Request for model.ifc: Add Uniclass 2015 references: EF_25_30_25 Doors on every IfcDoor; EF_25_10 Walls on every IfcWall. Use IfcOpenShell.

First a look at what the model holds.

```python
import ifcopenshell

model = ifcopenshell.open("model.ifc")
print(model.schema)
print("classifications:", [c.Name for c in model.by_type("IfcClassification")])
for ifc_class in ("IfcDoor", "IfcRoof", "IfcStair", "IfcWall", "IfcWindow"):
    print(ifc_class, len(model.by_type(ifc_class)))
```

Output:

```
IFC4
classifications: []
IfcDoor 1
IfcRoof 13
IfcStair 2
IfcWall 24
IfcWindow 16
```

```python
import ifcopenshell
import ifcopenshell.api.classification

model = ifcopenshell.open("model.ifc")

system = ifcopenshell.api.classification.add_classification(model, classification="Uniclass 2015")

codes = {
    "IfcDoor": ("EF_25_30_25", "Doors"),
    "IfcWall": ("EF_25_10", "Walls"),
}
for ifc_class, (code, name) in codes.items():
    products = model.by_type(ifc_class)
    ifcopenshell.api.classification.add_reference(
        model, products=products, classification=system, identification=code, name=name
    )
    print(code, len(products))

model.write("model-out.ifc")
```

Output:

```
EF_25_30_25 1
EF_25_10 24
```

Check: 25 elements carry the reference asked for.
